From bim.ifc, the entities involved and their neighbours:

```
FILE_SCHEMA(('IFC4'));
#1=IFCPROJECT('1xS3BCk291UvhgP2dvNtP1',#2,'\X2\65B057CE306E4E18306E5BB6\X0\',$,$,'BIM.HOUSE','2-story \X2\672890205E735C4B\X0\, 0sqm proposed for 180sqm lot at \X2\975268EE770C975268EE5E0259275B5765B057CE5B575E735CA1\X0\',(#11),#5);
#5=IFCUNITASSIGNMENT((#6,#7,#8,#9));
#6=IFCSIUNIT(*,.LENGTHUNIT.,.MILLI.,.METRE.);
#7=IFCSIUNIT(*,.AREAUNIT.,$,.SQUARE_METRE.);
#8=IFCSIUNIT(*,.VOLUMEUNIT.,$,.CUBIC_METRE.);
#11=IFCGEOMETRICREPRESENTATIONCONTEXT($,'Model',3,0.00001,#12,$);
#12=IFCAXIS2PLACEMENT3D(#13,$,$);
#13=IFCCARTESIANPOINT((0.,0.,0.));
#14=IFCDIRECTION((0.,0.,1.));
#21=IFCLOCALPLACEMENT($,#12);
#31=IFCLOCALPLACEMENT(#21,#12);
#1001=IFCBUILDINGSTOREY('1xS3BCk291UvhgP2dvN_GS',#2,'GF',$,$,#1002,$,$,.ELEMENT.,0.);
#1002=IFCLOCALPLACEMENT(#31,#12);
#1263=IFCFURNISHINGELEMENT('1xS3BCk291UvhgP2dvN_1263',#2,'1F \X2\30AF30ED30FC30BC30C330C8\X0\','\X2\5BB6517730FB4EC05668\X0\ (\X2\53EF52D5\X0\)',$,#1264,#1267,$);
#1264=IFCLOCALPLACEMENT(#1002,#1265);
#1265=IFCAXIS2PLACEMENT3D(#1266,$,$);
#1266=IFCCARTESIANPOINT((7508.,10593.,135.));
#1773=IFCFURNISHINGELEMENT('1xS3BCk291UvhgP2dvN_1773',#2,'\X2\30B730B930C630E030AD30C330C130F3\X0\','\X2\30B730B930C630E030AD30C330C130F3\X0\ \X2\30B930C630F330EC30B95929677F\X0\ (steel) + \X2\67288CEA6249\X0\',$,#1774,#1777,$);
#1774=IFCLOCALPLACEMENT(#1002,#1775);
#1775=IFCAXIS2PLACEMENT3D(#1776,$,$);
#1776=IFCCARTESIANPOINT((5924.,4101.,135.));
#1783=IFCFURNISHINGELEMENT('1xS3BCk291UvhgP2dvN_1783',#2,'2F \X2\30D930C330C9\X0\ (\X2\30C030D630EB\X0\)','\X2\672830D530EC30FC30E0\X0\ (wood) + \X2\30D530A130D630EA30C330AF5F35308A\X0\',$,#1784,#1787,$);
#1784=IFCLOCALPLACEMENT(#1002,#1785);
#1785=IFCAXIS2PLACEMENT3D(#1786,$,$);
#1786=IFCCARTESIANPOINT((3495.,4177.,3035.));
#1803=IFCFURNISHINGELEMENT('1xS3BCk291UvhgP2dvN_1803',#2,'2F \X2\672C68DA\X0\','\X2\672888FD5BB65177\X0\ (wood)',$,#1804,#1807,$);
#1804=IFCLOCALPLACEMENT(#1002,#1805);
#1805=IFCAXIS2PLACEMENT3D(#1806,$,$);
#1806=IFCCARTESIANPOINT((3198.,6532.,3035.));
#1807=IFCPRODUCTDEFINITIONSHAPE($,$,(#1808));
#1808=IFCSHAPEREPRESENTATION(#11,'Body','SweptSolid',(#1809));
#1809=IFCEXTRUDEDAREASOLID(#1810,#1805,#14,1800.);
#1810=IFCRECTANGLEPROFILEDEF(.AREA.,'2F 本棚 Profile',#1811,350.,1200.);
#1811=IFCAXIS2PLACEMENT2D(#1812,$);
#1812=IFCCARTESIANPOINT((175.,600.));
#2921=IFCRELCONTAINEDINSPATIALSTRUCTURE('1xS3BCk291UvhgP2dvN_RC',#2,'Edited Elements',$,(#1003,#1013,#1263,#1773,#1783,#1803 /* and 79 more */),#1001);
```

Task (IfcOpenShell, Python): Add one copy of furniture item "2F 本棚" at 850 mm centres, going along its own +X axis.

```python
import ifcopenshell
import ifcopenshell.api.geometry
import ifcopenshell.api.root
import ifcopenshell.util.element
import ifcopenshell.util.placement
import ifcopenshell.util.unit

model = ifcopenshell.open("bim.ifc")
unit_scale = ifcopenshell.util.unit.calculate_unit_scale(model)


def reuse_history(source, copy):
    """copy_class also copies each property set's owner history, people and application; keep the originals."""
    for rel in copy.IsDefinedBy:
        if rel.is_a("IfcRelDefinesByProperties") and (history := rel.RelatingPropertyDefinition.OwnerHistory):
            rel.RelatingPropertyDefinition.OwnerHistory = source.OwnerHistory
            ifcopenshell.util.element.remove_deep2(model, history)


source = model.by_id(1803)
base = ifcopenshell.util.placement.get_local_placement(source.ObjectPlacement)
step = base[:3, 0] * 0.85 / unit_scale

for i in range(1, 2):
    copy = ifcopenshell.api.root.copy_class(model, product=source)
    copy.Representation = ifcopenshell.util.element.copy_deep(
        model, source.Representation, exclude=["IfcGeometricRepresentationContext", "IfcRepresentationMap"]
    )
    reuse_history(source, copy)
    matrix = base.copy()
    matrix[:3, 3] += i * step
    print("added at", matrix[:3, 3].round(3) + 0.0)
    ifcopenshell.api.geometry.edit_object_placement(model, product=copy, matrix=matrix, is_si=False)

model.write("bim_edited.ifc")
```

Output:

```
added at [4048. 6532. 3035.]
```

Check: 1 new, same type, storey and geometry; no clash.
